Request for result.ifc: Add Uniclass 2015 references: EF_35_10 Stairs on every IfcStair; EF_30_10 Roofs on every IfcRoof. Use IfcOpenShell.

First a look at what the model holds.

```python
import ifcopenshell

model = ifcopenshell.open("result.ifc")
print(model.schema)
print("classifications:", [c.Name for c in model.by_type("IfcClassification")])
for ifc_class in ("IfcDoor", "IfcRoof", "IfcStair", "IfcWall", "IfcWindow"):
    print(ifc_class, len(model.by_type(ifc_class)))
```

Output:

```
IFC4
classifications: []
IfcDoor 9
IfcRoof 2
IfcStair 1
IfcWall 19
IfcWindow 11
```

```python
import ifcopenshell
import ifcopenshell.api.classification

model = ifcopenshell.open("result.ifc")

system = ifcopenshell.api.classification.add_classification(model, classification="Uniclass 2015")

codes = {
    "IfcStair": ("EF_35_10", "Stairs"),
    "IfcRoof": ("EF_30_10", "Roofs"),
}
for ifc_class, (code, name) in codes.items():
    products = model.by_type(ifc_class)
    ifcopenshell.api.classification.add_reference(
        model, products=products, classification=system, identification=code, name=name
    )
    print(code, len(products))

model.write("result_rev.ifc")
```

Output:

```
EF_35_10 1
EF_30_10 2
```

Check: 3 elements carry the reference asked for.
